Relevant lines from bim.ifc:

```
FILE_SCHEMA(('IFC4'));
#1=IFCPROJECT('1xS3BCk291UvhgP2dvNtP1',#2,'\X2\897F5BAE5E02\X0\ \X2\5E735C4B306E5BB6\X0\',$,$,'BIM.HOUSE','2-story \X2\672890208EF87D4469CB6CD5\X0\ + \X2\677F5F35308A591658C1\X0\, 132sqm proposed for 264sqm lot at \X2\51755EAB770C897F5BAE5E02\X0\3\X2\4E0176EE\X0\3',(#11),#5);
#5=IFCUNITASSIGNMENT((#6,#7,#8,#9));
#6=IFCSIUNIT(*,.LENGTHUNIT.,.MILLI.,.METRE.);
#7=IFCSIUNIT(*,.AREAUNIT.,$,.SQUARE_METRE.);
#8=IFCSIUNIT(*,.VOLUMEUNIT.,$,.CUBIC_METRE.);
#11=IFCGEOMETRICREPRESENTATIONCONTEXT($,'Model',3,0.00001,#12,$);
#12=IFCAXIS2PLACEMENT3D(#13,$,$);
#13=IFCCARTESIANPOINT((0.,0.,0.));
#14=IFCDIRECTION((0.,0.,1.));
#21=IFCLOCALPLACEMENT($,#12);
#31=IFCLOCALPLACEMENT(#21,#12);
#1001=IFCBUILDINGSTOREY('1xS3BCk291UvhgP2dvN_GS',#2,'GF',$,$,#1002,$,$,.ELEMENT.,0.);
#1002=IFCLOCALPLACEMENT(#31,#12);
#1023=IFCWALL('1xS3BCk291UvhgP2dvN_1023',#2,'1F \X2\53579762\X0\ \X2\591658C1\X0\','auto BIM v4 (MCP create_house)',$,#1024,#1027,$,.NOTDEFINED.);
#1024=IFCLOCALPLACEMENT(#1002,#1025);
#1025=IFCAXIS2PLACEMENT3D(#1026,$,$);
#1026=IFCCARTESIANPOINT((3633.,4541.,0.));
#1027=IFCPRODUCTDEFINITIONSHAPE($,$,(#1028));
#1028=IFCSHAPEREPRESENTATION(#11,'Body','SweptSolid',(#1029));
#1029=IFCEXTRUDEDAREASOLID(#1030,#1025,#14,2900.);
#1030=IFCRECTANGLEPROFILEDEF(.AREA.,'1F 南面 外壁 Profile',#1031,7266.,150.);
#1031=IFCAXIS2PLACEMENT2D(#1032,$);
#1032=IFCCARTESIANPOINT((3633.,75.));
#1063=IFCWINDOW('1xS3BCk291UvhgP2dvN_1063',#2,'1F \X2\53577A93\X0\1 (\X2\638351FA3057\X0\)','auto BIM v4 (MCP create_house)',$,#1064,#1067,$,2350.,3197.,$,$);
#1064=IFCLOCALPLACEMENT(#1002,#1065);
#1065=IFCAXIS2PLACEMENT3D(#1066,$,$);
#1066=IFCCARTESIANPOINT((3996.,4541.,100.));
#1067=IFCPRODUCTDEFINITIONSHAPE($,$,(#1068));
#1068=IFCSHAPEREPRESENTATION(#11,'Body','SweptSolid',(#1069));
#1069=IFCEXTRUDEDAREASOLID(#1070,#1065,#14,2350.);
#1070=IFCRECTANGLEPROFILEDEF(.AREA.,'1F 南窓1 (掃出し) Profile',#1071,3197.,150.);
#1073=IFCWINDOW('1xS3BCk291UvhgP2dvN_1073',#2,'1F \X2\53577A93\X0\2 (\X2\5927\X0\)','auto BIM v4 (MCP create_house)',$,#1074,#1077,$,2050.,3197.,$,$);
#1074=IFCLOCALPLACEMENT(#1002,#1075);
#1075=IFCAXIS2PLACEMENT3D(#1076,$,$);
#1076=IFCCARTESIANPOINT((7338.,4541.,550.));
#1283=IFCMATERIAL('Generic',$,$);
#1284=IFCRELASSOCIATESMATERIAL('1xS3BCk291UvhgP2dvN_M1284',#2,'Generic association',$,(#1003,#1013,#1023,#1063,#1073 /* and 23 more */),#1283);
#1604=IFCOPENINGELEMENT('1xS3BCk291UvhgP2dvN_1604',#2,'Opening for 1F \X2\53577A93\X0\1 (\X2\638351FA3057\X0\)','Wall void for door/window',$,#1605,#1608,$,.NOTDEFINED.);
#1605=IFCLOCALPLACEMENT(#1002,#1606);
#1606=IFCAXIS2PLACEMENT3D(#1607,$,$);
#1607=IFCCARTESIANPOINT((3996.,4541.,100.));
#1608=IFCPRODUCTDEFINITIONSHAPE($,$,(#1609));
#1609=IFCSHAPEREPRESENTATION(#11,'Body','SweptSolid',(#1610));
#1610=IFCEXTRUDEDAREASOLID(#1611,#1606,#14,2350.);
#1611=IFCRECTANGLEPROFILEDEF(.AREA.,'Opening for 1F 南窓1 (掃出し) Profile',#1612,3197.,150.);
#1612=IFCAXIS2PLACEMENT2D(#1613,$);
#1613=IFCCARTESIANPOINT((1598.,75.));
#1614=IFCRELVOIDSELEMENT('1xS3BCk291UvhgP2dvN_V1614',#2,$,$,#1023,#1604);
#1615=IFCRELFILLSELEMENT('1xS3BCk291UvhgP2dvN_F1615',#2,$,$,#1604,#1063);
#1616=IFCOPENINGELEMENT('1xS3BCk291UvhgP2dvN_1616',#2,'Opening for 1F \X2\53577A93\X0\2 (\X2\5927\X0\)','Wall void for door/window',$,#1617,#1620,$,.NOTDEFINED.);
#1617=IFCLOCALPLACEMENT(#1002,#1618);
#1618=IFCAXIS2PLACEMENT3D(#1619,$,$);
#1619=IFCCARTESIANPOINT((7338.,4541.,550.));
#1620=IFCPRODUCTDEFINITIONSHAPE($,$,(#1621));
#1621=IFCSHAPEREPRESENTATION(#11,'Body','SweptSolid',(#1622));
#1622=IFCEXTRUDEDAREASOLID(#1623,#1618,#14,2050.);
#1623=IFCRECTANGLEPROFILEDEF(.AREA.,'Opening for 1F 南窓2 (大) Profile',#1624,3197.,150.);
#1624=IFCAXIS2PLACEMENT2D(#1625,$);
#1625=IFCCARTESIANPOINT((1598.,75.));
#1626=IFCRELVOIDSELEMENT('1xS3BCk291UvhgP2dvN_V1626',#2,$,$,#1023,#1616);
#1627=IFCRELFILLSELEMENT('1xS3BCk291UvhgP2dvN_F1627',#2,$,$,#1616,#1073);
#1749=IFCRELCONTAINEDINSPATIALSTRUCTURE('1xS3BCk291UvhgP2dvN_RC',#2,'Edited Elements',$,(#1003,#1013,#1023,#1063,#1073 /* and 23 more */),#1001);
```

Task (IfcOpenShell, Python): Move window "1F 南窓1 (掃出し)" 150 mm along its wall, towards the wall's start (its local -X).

```python
import ifcopenshell
import ifcopenshell.api.geometry
import ifcopenshell.util.placement

model = ifcopenshell.open("bim.ifc")

window = model.by_id(1063)
opening = window.FillsVoids[0].RelatingOpeningElement
wall = opening.VoidsElements[0].RelatingBuildingElement

wall_matrix = ifcopenshell.util.placement.get_local_placement(wall.ObjectPlacement)
shift = wall_matrix[:3, 0] * -150.0
before = ifcopenshell.util.placement.get_local_placement(window.ObjectPlacement)[:3, 3].copy()

# The window is not placed relative to its opening, so move both.
for product in (opening, window):
    matrix = ifcopenshell.util.placement.get_local_placement(product.ObjectPlacement)
    matrix[:3, 3] += shift
    ifcopenshell.api.geometry.edit_object_placement(model, product=product, matrix=matrix, is_si=False)

after = ifcopenshell.util.placement.get_local_placement(window.ObjectPlacement)[:3, 3]
print("window moved by", (after - before).round(3) + 0.0)

model.write("bim_updated.ifc")
```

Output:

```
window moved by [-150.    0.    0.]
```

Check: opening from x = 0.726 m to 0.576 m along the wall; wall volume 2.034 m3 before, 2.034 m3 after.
